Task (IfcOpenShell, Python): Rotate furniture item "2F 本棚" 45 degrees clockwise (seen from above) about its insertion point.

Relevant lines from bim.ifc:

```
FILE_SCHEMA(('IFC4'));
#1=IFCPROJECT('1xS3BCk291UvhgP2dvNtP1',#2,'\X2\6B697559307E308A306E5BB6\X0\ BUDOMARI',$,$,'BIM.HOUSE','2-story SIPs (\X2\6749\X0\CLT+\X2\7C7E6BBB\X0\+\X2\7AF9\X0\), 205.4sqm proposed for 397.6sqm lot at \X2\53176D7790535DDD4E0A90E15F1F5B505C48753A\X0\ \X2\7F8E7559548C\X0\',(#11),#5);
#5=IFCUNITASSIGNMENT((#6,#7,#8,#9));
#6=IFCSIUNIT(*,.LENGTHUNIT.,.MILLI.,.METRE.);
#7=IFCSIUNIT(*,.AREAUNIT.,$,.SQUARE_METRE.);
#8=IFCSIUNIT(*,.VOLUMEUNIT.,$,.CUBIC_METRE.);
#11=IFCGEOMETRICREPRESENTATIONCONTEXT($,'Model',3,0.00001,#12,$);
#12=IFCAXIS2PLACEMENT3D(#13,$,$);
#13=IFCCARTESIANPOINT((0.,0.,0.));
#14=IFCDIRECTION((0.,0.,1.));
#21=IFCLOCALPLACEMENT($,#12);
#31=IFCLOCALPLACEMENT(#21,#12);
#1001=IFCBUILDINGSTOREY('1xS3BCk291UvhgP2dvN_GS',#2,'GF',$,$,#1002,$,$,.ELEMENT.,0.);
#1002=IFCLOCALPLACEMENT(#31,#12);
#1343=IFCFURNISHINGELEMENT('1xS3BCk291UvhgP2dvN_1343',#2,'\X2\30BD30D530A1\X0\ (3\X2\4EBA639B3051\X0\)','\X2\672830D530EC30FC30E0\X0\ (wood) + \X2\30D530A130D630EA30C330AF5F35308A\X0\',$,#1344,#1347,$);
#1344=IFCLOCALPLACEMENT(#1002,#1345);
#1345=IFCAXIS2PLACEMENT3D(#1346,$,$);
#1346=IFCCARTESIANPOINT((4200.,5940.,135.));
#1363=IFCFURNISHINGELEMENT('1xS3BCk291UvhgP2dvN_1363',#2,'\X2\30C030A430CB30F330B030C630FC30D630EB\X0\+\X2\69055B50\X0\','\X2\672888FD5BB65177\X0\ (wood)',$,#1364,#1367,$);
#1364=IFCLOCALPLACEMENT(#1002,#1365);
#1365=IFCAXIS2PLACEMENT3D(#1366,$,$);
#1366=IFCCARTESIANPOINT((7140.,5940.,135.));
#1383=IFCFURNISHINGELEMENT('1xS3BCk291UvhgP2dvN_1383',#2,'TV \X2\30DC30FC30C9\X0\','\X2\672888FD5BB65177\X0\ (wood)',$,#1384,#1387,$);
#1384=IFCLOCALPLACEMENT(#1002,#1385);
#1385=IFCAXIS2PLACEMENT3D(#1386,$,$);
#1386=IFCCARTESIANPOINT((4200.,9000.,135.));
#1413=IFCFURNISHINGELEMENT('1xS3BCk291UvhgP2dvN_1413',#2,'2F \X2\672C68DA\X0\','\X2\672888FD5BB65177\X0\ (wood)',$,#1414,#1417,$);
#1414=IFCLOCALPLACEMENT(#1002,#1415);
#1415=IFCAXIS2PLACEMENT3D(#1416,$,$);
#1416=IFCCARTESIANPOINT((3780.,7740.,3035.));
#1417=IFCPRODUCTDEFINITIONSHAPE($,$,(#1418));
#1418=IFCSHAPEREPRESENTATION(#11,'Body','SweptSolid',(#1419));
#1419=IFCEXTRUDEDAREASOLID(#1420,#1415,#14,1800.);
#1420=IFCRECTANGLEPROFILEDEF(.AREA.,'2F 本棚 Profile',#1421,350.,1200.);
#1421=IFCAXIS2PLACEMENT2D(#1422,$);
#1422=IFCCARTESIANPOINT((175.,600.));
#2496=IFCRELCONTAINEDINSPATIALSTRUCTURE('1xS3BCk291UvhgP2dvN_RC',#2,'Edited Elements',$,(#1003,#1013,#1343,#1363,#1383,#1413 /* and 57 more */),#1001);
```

```python
import ifcopenshell
import ifcopenshell.api.geometry
import ifcopenshell.util.placement

model = ifcopenshell.open("bim.ifc")

item = model.by_guid("1xS3BCk291UvhgP2dvN_1413")
matrix = ifcopenshell.util.placement.get_local_placement(item.ObjectPlacement)
matrix = matrix @ ifcopenshell.util.placement.rotation(-45, "Z")
ifcopenshell.api.geometry.edit_object_placement(model, product=item, matrix=matrix, is_si=False)

print(ifcopenshell.util.placement.get_local_placement(item.ObjectPlacement).round(3) + 0.0)

model.write("bim-out.ifc")
```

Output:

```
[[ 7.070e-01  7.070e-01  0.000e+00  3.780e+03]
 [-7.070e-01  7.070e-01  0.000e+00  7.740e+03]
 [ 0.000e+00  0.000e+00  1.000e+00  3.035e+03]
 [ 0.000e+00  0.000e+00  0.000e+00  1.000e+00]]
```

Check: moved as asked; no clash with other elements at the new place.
